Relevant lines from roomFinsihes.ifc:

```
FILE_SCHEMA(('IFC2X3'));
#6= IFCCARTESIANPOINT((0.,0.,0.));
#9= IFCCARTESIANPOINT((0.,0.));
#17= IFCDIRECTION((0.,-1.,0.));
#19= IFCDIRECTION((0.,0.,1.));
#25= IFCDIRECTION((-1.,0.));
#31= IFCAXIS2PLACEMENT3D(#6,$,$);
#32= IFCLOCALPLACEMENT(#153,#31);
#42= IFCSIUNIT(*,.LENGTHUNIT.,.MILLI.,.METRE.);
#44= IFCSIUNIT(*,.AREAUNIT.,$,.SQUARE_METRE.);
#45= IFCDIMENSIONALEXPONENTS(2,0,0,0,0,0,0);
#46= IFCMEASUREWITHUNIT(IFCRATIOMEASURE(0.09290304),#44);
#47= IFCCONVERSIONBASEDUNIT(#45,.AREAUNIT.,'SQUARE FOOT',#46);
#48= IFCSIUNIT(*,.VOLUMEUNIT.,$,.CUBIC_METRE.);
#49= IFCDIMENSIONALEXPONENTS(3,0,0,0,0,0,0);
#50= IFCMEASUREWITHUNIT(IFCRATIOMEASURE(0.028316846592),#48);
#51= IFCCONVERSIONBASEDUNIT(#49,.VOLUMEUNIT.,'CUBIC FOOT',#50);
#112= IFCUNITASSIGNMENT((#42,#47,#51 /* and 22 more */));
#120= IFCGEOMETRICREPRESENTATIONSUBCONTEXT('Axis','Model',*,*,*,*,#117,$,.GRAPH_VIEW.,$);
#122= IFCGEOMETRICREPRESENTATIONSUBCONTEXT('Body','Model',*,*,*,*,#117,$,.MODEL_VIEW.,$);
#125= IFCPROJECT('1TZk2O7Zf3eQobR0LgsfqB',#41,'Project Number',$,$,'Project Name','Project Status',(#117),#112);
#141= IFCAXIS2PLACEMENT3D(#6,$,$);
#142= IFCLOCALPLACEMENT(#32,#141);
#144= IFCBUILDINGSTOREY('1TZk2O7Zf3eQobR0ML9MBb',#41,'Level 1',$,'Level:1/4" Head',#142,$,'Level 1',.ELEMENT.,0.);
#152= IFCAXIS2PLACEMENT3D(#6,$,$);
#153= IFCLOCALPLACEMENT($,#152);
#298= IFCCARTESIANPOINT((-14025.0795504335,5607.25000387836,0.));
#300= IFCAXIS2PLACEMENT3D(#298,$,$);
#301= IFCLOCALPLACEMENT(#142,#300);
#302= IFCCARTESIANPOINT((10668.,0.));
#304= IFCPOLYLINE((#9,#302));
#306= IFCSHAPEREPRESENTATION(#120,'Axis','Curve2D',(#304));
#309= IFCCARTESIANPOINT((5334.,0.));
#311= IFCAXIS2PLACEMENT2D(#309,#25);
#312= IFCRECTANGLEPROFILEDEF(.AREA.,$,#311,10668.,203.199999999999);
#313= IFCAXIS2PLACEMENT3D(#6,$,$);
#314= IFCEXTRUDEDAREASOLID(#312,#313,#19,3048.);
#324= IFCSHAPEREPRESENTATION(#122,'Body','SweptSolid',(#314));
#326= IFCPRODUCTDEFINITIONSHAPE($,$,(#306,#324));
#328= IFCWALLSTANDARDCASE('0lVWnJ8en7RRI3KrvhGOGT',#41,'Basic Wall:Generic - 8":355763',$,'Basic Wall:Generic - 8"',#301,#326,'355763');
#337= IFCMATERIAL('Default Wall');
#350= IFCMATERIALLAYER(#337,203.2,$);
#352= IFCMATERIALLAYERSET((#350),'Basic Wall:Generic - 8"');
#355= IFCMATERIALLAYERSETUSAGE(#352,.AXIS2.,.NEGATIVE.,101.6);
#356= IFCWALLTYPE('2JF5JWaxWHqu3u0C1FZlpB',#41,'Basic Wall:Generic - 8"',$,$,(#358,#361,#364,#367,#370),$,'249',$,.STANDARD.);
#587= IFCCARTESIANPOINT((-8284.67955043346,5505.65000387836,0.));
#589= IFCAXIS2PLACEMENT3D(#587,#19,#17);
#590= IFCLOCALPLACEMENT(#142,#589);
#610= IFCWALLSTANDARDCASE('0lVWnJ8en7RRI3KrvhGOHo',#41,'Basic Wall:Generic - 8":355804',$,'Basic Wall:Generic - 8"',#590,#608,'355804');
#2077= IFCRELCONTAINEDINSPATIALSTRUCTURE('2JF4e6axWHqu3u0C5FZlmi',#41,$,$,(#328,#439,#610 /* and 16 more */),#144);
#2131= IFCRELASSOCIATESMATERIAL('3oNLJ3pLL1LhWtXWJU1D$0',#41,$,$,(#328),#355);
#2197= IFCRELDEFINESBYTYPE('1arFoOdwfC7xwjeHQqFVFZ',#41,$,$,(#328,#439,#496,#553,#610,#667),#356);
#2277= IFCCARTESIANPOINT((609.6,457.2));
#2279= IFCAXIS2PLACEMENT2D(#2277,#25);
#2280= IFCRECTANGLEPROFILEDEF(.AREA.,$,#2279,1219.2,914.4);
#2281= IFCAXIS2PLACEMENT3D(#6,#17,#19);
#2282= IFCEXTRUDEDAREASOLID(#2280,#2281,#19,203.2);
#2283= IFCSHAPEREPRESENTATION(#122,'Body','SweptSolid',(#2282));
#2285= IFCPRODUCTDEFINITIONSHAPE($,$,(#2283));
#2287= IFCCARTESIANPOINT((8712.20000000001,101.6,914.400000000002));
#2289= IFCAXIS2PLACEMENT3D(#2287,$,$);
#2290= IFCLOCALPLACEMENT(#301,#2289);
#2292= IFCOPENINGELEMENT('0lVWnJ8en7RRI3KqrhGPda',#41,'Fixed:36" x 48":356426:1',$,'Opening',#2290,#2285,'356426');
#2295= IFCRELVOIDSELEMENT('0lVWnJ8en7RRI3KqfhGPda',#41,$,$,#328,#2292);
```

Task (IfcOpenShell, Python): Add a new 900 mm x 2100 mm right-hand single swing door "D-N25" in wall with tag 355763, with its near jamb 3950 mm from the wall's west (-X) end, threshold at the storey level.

```python
import numpy as np
import ifcopenshell
import ifcopenshell.api.feature
import ifcopenshell.api.geometry
import ifcopenshell.api.root
import ifcopenshell.api.spatial
import ifcopenshell.api.type
import ifcopenshell.geom
import ifcopenshell.util.element
import ifcopenshell.util.placement
import ifcopenshell.util.representation
import ifcopenshell.util.shape
import ifcopenshell.util.unit

model = ifcopenshell.open("roomFinsihes.ifc")
unit_scale = ifcopenshell.util.unit.calculate_unit_scale(model)
settings = ifcopenshell.geom.settings()


def volume(element):
    """Net volume in cubic metres, openings subtracted."""
    shape = ifcopenshell.geom.create_shape(settings, element)
    return ifcopenshell.util.shape.get_volume(shape.geometry)


wall = model.by_guid("0lVWnJ8en7RRI3KrvhGOGT")
storey = ifcopenshell.util.element.get_container(wall, ifc_class="IfcBuildingStorey")
context = ifcopenshell.util.representation.get_context(model, "Model", "Body", "MODEL_VIEW")
before = volume(wall)

width, height, from_end, sill = 0.9, 2.1, 3.95, 0.0  # metres

# The wall runs along its own X axis, and the end named is its -X end.
wall_shape = ifcopenshell.geom.create_shape(settings, wall)
x, y, z = ifcopenshell.util.shape.get_vertices(wall_shape.geometry).T
start = x.min() + from_end
face, thickness = float(y.min()), float(y.max() - y.min())
wall_matrix = ifcopenshell.util.placement.get_local_placement(wall.ObjectPlacement)
level = ifcopenshell.util.placement.get_local_placement(storey.ObjectPlacement)[2, 3]


def in_wall(x, y):
    """Placement at x, y metres in the wall's axes, at sill height."""
    matrix = wall_matrix.copy()
    matrix[:, 3] = wall_matrix @ np.array([x / unit_scale, y / unit_scale, 0.0, 1.0])
    matrix[2, 3] = level + sill / unit_scale
    return matrix


# Opening: a box that overshoots both wall faces by 50 mm.
opening = ifcopenshell.api.root.create_entity(model, ifc_class="IfcOpeningElement")
box = ifcopenshell.api.geometry.add_wall_representation(
    model, context=context, length=width, height=height, thickness=thickness + 0.1
)
ifcopenshell.api.geometry.assign_representation(model, product=opening, representation=box)
ifcopenshell.api.geometry.edit_object_placement(model, product=opening, matrix=in_wall(start, face - 0.05), is_si=False)
ifcopenshell.api.feature.add_feature(model, feature=opening, element=wall)

door = ifcopenshell.api.root.create_entity(model, ifc_class="IfcDoor", name="D-N25")
door.OverallWidth, door.OverallHeight = width / unit_scale, height / unit_scale
body = ifcopenshell.api.geometry.add_door_representation(
    model,
    context=context,
    overall_width=door.OverallWidth,
    overall_height=door.OverallHeight,
    operation_type="SINGLE_SWING_RIGHT",
    lining_properties={"LiningDepth": thickness / unit_scale, "ThresholdDepth": thickness / unit_scale},
)
ifcopenshell.api.geometry.assign_representation(model, product=door, representation=body)
ifcopenshell.api.spatial.assign_container(model, products=[door], relating_structure=storey)
fills = ifcopenshell.api.feature.add_filling(model, opening=opening, element=door)
fills.OwnerHistory = door.OwnerHistory  # required in IFC2X3

# IFC2X3 keeps the operation on the door style.
style = ifcopenshell.api.root.create_entity(model, ifc_class="IfcDoorStyle", name="D-N25")
style.OperationType, style.ConstructionType = "SINGLE_SWING_RIGHT", "NOTDEFINED"
style.ParameterTakesPrecedence = style.Sizeable = False
ifcopenshell.api.type.assign_type(model, related_objects=[door], relating_type=style)

# The lining spans the wall, so the door starts at the wall face.
ifcopenshell.api.geometry.edit_object_placement(model, product=door, matrix=in_wall(start, face), is_si=False)

after = volume(wall)

print(f"wall volume {before:.3f} -> {after:.3f} m3")

model.write("roomFinsihes_rev.ifc")
```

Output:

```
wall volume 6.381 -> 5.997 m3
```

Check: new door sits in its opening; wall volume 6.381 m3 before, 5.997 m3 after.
